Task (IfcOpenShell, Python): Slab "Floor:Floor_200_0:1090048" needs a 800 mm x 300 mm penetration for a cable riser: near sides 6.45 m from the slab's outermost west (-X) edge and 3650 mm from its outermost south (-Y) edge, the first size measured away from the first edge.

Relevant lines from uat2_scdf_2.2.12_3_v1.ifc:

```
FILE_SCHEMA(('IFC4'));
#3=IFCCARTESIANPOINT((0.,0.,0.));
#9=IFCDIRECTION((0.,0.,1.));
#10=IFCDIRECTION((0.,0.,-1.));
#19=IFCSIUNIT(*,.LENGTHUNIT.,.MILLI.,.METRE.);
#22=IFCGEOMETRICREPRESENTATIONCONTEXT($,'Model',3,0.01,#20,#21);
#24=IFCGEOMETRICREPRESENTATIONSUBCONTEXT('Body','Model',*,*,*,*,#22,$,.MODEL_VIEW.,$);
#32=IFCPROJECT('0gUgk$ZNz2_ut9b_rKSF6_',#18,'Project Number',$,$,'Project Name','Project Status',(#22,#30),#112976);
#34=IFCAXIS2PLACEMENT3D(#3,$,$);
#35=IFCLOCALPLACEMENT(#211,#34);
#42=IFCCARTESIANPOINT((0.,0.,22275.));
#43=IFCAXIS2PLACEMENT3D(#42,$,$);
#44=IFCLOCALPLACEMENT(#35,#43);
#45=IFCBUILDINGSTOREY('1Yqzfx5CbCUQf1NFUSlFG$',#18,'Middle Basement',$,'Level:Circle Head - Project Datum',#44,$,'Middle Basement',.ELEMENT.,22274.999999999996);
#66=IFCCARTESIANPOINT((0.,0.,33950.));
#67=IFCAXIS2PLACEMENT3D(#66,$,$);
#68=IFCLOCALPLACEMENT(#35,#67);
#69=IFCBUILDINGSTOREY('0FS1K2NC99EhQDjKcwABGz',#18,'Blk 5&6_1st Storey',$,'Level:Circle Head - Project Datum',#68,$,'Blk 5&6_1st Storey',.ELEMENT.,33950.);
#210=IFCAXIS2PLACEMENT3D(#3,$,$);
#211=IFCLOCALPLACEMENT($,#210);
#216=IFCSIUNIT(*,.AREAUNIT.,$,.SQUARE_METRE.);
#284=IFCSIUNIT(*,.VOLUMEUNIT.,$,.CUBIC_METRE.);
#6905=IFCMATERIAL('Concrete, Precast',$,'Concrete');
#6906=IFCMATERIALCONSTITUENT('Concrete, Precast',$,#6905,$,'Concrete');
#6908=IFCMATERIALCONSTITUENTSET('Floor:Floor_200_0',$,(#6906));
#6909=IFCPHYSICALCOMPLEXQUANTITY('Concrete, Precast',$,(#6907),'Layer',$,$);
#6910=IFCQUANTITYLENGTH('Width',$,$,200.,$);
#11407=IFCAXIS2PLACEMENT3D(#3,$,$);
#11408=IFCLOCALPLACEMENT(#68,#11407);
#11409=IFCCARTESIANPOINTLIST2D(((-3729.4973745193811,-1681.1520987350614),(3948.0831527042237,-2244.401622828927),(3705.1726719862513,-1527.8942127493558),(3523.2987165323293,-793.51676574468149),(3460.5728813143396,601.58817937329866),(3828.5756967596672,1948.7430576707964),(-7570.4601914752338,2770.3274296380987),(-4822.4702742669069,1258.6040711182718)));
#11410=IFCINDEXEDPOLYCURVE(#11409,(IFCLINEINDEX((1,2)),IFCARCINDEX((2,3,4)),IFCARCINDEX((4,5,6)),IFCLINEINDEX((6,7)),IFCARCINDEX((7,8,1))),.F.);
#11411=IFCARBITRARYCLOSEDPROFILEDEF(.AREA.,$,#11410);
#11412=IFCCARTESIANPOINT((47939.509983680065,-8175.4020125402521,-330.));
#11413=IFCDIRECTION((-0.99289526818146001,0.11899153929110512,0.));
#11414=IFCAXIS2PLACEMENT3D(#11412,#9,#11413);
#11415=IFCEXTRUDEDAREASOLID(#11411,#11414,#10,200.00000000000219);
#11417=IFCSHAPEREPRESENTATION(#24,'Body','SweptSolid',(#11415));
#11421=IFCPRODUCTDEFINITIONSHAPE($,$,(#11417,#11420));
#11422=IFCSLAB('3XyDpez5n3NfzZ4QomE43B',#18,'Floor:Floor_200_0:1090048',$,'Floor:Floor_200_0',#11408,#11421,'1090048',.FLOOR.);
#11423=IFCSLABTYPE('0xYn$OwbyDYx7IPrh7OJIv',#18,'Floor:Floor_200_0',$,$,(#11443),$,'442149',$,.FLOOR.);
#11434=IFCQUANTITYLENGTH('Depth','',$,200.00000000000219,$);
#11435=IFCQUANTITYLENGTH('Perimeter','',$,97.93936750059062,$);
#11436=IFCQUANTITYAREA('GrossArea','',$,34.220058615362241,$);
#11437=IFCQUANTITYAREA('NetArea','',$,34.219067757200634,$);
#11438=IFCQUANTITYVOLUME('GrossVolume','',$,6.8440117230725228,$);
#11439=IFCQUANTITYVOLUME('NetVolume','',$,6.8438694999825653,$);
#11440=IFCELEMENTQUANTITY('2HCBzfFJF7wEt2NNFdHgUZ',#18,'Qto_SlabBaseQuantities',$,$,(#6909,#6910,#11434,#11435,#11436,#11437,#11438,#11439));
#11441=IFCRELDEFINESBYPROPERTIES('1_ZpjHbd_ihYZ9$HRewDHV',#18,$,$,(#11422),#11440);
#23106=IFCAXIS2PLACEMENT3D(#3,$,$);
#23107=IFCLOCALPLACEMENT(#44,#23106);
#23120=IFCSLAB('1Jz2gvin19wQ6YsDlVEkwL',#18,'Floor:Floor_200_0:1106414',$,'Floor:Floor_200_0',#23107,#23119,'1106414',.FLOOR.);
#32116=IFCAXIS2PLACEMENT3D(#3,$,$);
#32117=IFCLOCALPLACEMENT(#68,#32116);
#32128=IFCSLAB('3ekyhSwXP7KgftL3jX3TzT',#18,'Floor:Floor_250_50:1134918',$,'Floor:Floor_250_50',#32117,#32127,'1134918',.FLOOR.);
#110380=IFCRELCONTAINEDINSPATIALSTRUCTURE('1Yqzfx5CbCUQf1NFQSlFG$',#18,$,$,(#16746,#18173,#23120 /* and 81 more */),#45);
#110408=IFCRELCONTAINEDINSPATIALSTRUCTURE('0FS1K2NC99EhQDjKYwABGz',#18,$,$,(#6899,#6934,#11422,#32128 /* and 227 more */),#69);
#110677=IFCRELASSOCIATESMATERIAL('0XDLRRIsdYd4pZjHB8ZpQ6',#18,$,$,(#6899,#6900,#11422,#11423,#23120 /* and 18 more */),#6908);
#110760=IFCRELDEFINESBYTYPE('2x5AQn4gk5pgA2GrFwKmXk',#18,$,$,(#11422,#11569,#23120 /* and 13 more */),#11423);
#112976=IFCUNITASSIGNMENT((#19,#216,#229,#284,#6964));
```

```python
import numpy as np
import ifcopenshell
import ifcopenshell.api.feature
import ifcopenshell.api.geometry
import ifcopenshell.api.pset
import ifcopenshell.api.root
import ifcopenshell.geom
import ifcopenshell.util.element
import ifcopenshell.util.placement
import ifcopenshell.util.representation
import ifcopenshell.util.shape
import ifcopenshell.util.unit

model = ifcopenshell.open("uat2_scdf_2.2.12_3_v1.ifc")
unit_scale = ifcopenshell.util.unit.calculate_unit_scale(model)
area_scale = ifcopenshell.util.unit.calculate_unit_scale(model, "AREAUNIT")
volume_scale = ifcopenshell.util.unit.calculate_unit_scale(model, "VOLUMEUNIT")
settings = ifcopenshell.geom.settings()


def volume(element):
    """Net volume in cubic metres, openings subtracted."""
    shape = ifcopenshell.geom.create_shape(settings, element)
    return ifcopenshell.util.shape.get_volume(shape.geometry)


slab = model.by_guid("3XyDpez5n3NfzZ4QomE43B")
before = volume(slab)

# Extent in the slab's own axes, in metres. The edges named are its -X and -Y sides.
slab_shape = ifcopenshell.geom.create_shape(settings, slab)
vertices = ifcopenshell.util.shape.get_vertices(slab_shape.geometry)
x_min, y_min, bottom = vertices.min(axis=0)
top = vertices[:, 2].max()

opening = ifcopenshell.api.root.create_entity(model, ifc_class="IfcOpeningElement", name="Cable riser opening", predefined_type="OPENING")
context = ifcopenshell.util.representation.get_context(model, "Model", "Body", "MODEL_VIEW")
width, depth = 0.8, 0.3
outline = [(0.0, 0.0), (width, 0.0), (width, depth), (0.0, depth), (0.0, 0.0)]
# Overshoot both faces by 50 mm so the cut is clean.
shape = ifcopenshell.api.geometry.add_slab_representation(
    model, context=context, depth=top - bottom + 0.1, polyline=outline
)
ifcopenshell.api.geometry.assign_representation(model, product=opening, representation=shape)

matrix = ifcopenshell.util.placement.get_local_placement(slab.ObjectPlacement)
matrix[:, 3] = matrix @ np.append(np.array([x_min + 6.45, y_min + 3.65, bottom - 0.05]) / unit_scale, 1.0)
ifcopenshell.api.geometry.edit_object_placement(model, product=opening, matrix=matrix, is_si=False)
ifcopenshell.api.feature.add_feature(model, feature=opening, element=slab)

after = volume(slab)

# Update the slab's stored quantities.
qto = model.by_id(ifcopenshell.util.element.get_pset(slab, "Qto_SlabBaseQuantities", should_inherit=False)["id"])
ifcopenshell.api.pset.edit_qto(model, qto=qto, properties={
    "NetArea": after / (top - bottom) / area_scale,
    "NetVolume": after / volume_scale,
})

print(f"slab volume {before:.3f} -> {after:.3f} m3")

model.write("uat2_scdf_2.2.12_3_v1_rev.ifc")
```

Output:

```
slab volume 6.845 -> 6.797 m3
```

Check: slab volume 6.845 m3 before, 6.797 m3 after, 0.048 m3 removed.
